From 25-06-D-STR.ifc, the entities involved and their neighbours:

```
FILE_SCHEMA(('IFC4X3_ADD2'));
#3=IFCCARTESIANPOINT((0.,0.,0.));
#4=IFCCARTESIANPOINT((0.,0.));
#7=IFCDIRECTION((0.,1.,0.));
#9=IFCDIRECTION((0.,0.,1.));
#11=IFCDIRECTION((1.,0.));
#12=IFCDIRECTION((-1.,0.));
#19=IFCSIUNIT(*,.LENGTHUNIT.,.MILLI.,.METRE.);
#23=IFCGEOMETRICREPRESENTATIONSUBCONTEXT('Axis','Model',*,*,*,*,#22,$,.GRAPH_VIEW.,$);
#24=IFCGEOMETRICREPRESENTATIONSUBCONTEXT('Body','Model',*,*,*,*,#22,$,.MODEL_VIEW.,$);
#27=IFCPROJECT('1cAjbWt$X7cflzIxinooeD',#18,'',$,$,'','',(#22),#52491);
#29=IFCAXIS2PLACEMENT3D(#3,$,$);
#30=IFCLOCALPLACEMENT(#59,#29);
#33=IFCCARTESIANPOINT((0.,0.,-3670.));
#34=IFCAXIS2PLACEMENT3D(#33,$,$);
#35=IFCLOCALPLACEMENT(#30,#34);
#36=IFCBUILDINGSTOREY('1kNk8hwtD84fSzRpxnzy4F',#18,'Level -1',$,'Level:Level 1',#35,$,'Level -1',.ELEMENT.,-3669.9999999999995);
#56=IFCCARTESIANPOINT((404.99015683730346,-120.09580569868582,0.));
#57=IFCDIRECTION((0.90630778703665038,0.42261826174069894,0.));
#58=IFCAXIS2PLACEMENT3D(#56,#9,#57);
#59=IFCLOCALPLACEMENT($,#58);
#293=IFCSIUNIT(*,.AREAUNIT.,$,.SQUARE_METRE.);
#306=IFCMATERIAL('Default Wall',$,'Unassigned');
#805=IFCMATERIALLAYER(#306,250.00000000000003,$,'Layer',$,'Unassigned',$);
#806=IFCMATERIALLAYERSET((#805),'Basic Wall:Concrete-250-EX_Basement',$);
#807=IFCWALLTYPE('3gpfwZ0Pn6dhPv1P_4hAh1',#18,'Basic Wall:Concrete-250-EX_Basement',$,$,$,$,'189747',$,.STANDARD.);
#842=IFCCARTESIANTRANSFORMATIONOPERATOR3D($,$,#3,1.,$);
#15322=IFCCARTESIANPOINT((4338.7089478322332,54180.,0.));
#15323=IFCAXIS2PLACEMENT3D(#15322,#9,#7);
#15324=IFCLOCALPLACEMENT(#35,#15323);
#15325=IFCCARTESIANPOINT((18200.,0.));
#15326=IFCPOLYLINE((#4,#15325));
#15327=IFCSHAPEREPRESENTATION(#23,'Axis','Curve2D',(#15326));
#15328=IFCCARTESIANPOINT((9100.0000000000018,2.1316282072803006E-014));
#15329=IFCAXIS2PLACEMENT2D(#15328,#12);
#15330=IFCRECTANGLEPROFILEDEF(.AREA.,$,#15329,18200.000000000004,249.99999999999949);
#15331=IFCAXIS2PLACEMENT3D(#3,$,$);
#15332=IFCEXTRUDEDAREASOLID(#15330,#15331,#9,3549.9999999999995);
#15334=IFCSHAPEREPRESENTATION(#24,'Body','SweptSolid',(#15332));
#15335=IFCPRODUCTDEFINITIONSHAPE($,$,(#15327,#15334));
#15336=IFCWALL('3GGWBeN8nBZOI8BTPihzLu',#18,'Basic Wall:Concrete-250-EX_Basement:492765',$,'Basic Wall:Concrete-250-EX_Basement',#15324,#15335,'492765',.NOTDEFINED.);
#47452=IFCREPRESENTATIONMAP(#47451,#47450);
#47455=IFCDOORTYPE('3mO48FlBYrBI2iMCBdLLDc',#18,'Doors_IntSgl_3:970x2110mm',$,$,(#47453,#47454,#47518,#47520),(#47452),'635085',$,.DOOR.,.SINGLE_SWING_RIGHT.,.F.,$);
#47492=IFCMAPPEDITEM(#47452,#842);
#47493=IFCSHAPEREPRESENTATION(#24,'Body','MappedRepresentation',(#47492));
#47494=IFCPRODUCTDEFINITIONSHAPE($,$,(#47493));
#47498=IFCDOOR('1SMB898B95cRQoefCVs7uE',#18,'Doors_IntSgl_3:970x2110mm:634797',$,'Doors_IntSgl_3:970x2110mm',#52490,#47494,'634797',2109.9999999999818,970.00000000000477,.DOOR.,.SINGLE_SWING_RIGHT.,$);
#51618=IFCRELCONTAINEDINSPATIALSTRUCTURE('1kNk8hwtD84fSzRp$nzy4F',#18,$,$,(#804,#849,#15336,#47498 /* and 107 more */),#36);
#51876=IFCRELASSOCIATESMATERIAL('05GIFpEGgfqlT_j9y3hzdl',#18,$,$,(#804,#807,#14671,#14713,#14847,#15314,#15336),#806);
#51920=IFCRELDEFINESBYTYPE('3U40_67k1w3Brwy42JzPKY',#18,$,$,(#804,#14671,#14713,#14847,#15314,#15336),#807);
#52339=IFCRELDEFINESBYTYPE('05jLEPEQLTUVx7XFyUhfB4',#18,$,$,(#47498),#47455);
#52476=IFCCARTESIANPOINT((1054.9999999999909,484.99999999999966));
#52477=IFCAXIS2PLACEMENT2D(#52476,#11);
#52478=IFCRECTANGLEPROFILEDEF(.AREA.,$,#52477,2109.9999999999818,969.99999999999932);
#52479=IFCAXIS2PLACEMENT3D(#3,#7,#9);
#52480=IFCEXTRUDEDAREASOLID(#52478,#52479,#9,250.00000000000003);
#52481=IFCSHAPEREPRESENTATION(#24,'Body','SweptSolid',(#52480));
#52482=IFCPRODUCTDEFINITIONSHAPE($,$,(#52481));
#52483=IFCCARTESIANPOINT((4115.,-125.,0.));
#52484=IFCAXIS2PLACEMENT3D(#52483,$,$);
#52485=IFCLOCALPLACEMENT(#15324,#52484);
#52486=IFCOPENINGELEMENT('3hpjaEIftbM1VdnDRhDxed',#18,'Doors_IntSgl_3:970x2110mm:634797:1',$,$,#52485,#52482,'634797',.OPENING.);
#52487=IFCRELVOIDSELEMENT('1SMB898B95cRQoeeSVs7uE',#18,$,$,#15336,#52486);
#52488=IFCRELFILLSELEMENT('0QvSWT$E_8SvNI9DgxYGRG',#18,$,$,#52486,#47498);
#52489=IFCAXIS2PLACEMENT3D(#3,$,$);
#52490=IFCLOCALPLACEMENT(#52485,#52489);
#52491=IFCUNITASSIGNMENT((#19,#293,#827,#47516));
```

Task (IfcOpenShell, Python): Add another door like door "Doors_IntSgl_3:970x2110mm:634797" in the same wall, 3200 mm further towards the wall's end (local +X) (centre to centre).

```python
import ifcopenshell
import ifcopenshell.api.feature
import ifcopenshell.api.geometry
import ifcopenshell.api.root
import ifcopenshell.geom
import ifcopenshell.util.element
import ifcopenshell.util.placement
import ifcopenshell.util.shape

model = ifcopenshell.open("25-06-D-STR.ifc")
settings = ifcopenshell.geom.settings()


def volume(element):
    """Net volume in cubic metres, openings subtracted."""
    shape = ifcopenshell.geom.create_shape(settings, element)
    return ifcopenshell.util.shape.get_volume(shape.geometry)


def reuse_history(source, copy):
    """copy_class also copies each property set's owner history, people and application; keep the originals."""
    for rel in copy.IsDefinedBy:
        if rel.is_a("IfcRelDefinesByProperties") and (history := rel.RelatingPropertyDefinition.OwnerHistory):
            rel.RelatingPropertyDefinition.OwnerHistory = source.OwnerHistory
            ifcopenshell.util.element.remove_deep2(model, history)


door = model.by_guid("1SMB898B95cRQoefCVs7uE")
opening = door.FillsVoids[0].RelatingOpeningElement
wall = opening.VoidsElements[0].RelatingBuildingElement
before = volume(wall)
shift = ifcopenshell.util.placement.get_local_placement(wall.ObjectPlacement)[:3, 0] * 3200.0

# copy_class copies the void relationship, type, container and properties, but no geometry.
new_opening = ifcopenshell.api.root.copy_class(model, product=opening)
new_opening.Representation = ifcopenshell.util.element.copy_deep(
    model, opening.Representation, exclude=["IfcGeometricRepresentationContext", "IfcRepresentationMap"]
)
new_opening.Name = "Doors_IntSgl_3:970x2110mm"
new_opening.Tag = None
new_door = ifcopenshell.api.root.copy_class(model, product=door)
new_door.Representation = ifcopenshell.util.element.copy_deep(
    model, door.Representation, exclude=["IfcGeometricRepresentationContext", "IfcRepresentationMap"]
)
new_door.Name = "Doors_IntSgl_3:970x2110mm"
new_door.Tag = None
reuse_history(door, new_door)
ifcopenshell.api.feature.add_filling(model, opening=new_opening, element=new_door)

for old, new in ((opening, new_opening), (door, new_door)):
    matrix = ifcopenshell.util.placement.get_local_placement(old.ObjectPlacement)
    matrix[:3, 3] += shift
    ifcopenshell.api.geometry.edit_object_placement(model, product=new, matrix=matrix, is_si=False)

after = volume(wall)

print(f"wall volume {before:.3f} -> {after:.3f} m3")

model.write("25-06-D-STR_rev.ifc")
```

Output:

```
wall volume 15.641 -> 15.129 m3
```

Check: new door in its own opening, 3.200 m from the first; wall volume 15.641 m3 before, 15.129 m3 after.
